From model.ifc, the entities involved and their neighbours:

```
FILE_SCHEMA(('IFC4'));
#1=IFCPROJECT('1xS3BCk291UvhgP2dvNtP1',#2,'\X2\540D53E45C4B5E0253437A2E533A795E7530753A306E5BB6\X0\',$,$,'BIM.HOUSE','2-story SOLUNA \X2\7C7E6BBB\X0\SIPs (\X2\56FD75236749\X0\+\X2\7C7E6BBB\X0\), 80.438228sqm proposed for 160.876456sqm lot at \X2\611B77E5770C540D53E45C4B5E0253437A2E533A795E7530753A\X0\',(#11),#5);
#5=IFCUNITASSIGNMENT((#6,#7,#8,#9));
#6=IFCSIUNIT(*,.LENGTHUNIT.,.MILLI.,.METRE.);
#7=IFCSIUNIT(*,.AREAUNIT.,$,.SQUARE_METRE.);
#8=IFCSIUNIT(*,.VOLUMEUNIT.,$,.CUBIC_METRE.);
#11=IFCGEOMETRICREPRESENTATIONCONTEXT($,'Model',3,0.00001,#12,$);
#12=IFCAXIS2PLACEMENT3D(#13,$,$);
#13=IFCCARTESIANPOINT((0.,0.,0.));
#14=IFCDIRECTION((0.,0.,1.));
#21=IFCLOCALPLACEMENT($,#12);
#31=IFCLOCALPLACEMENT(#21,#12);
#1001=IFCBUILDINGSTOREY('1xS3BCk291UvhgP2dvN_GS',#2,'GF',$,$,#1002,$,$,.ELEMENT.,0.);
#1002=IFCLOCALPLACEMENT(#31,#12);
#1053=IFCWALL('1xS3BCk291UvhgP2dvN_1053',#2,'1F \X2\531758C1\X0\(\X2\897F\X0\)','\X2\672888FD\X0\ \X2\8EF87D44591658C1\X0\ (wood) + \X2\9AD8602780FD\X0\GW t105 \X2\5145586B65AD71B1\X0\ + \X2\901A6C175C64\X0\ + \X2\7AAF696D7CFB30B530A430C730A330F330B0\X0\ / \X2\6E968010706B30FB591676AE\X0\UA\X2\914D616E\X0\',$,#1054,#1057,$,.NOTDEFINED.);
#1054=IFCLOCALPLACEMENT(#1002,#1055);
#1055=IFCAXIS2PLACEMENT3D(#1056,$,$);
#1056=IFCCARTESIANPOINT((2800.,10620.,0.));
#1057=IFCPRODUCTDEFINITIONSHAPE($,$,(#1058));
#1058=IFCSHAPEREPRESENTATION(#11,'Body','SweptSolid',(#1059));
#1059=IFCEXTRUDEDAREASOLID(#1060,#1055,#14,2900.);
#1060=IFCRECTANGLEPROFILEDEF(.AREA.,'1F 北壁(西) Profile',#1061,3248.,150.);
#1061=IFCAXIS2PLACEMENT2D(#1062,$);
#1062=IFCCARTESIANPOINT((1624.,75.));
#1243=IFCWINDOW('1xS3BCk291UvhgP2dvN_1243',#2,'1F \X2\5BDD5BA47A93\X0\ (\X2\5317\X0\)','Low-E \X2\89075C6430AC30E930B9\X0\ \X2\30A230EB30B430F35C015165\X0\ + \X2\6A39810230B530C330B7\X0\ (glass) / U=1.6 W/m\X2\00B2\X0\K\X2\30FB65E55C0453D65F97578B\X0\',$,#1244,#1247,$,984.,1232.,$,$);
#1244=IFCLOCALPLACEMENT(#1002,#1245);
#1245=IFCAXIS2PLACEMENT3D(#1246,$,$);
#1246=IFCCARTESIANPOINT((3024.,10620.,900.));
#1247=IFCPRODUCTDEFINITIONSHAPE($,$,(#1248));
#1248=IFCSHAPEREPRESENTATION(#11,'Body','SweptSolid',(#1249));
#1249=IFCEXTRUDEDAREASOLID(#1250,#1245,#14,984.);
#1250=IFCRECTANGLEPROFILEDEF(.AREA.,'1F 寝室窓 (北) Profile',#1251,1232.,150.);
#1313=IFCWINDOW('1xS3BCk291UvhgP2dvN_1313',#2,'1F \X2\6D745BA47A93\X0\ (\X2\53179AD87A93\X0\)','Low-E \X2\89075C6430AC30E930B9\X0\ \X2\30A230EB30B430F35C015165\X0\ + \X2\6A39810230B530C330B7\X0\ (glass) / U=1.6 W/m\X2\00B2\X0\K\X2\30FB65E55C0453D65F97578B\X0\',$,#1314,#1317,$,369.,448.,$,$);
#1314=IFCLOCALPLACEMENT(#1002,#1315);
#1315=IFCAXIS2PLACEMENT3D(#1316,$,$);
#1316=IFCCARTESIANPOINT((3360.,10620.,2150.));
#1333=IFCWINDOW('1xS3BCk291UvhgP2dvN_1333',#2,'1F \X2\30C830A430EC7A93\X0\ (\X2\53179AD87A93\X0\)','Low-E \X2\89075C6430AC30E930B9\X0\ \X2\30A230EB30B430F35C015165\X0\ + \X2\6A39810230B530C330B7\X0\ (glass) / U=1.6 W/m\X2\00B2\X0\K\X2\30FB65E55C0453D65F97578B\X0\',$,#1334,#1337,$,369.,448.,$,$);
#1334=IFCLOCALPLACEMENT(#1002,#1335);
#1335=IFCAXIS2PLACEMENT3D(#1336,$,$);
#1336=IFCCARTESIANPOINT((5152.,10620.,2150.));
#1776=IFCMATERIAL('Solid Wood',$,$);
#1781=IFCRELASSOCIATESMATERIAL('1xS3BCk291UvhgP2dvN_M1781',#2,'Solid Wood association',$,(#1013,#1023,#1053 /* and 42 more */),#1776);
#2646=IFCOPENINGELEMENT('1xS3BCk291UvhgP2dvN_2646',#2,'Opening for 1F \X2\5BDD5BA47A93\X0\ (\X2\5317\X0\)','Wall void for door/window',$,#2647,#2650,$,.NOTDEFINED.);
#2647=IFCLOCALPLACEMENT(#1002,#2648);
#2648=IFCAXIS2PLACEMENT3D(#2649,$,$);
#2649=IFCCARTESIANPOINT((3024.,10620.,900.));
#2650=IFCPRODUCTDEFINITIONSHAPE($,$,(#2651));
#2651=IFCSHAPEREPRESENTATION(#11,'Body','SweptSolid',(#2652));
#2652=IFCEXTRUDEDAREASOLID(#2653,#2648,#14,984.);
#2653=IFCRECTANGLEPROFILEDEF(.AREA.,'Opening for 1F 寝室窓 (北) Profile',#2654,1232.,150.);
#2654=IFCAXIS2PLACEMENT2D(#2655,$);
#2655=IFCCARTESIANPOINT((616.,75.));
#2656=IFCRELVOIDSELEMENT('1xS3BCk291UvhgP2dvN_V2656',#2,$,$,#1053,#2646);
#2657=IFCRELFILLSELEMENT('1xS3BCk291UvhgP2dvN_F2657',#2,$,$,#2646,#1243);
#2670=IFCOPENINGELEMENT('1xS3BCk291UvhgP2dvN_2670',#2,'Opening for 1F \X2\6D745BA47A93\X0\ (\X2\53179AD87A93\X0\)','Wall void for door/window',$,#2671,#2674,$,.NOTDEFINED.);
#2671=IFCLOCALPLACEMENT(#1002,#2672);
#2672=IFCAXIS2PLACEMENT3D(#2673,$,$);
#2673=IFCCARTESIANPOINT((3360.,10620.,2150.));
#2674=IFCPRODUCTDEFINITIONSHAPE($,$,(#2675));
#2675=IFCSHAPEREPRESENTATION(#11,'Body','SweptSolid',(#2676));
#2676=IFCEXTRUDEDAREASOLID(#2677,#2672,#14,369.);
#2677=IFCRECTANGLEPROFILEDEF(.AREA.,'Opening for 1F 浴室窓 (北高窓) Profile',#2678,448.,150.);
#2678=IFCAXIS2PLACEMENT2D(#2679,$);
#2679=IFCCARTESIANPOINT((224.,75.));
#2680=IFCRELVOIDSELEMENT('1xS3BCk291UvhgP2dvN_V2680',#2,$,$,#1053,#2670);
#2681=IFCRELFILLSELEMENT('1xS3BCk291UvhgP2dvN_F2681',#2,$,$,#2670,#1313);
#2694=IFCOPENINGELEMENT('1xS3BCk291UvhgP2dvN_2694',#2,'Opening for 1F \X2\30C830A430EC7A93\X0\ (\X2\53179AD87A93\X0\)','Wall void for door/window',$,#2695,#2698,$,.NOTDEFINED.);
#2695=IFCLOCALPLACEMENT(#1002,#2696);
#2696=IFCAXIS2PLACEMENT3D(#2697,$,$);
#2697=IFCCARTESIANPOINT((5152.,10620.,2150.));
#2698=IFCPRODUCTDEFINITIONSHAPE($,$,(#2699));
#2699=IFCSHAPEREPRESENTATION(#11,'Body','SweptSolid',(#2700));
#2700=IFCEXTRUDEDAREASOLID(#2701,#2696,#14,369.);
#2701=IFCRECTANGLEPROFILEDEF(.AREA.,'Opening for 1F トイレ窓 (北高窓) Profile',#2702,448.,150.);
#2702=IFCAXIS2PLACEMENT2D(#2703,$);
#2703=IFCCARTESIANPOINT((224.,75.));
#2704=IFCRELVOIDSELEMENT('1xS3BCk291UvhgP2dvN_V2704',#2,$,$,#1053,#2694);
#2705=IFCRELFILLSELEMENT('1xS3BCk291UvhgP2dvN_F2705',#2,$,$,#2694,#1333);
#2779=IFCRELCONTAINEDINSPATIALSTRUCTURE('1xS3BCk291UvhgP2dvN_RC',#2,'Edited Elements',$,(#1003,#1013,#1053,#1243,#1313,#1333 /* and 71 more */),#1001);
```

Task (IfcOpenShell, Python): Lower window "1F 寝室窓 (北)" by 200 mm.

```python
import numpy as np
import ifcopenshell
import ifcopenshell.api.geometry
import ifcopenshell.util.placement
import ifcopenshell.util.unit

model = ifcopenshell.open("model.ifc")
unit_scale = ifcopenshell.util.unit.calculate_unit_scale(model)

window = model.by_guid("1xS3BCk291UvhgP2dvN_1243")
opening = window.FillsVoids[0].RelatingOpeningElement
dz = -200.0

shift = np.array([0.0, 0.0, dz])
# The window is not placed relative to its opening, so move both.
for product in (opening, window):
    matrix = ifcopenshell.util.placement.get_local_placement(product.ObjectPlacement)
    matrix[:3, 3] += shift
    ifcopenshell.api.geometry.edit_object_placement(model, product=product, matrix=matrix, is_si=False)

print(f"moved by {dz * unit_scale:+.3f} m")

model.write("model-out.ifc")
```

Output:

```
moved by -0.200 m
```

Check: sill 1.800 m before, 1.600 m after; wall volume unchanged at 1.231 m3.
